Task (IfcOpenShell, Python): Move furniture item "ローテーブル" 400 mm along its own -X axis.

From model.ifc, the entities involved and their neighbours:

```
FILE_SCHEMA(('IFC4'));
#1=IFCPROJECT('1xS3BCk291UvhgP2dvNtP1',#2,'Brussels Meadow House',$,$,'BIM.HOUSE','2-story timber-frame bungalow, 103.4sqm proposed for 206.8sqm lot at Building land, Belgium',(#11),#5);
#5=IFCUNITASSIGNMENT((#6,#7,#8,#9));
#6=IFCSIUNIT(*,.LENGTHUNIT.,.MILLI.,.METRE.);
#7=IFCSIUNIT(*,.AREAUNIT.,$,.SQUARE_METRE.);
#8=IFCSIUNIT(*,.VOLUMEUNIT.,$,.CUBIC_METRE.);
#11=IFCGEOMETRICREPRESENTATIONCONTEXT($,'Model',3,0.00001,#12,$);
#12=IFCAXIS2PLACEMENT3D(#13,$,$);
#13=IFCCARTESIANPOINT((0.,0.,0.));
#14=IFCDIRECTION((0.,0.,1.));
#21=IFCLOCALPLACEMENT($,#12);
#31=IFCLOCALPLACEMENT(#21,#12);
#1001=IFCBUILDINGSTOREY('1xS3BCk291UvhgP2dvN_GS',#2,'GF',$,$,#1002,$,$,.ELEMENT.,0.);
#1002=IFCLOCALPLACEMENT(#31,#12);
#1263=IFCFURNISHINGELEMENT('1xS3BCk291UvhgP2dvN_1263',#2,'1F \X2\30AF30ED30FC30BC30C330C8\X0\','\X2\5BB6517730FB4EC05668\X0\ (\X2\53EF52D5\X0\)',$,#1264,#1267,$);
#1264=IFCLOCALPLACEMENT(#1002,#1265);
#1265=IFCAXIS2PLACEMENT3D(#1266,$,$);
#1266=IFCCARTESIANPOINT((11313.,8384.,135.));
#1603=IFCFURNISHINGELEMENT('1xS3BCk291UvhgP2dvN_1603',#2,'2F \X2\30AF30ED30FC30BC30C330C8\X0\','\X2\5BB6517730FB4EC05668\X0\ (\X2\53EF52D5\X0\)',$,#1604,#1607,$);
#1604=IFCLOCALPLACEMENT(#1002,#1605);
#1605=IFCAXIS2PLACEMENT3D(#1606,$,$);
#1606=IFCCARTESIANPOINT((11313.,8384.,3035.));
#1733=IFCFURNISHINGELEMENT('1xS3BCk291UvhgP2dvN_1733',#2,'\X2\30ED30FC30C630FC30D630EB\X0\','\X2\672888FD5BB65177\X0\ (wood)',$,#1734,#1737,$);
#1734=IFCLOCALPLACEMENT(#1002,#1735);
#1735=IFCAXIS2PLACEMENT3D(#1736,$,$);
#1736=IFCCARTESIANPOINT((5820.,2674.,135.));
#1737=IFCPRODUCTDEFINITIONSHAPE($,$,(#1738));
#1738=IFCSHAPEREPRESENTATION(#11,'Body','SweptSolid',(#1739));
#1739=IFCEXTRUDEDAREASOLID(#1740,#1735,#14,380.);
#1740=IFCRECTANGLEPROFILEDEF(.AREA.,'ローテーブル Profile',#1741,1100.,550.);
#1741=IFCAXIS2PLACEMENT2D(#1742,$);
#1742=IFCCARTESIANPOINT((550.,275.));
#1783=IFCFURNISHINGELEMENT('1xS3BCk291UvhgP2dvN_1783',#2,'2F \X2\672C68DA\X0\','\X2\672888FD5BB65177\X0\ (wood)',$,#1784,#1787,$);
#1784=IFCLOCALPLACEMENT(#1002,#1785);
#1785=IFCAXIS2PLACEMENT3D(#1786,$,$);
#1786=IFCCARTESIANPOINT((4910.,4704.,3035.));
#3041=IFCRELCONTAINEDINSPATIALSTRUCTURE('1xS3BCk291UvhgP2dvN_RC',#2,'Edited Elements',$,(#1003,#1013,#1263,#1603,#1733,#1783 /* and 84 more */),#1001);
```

```python
import ifcopenshell
import ifcopenshell.api.geometry
import ifcopenshell.util.placement

model = ifcopenshell.open("model.ifc")

item = model.by_guid("1xS3BCk291UvhgP2dvN_1733")
matrix = ifcopenshell.util.placement.get_local_placement(item.ObjectPlacement)
matrix[:3, 3] -= matrix[:3, 0] * 400.0
ifcopenshell.api.geometry.edit_object_placement(model, product=item, matrix=matrix, is_si=False)

print(ifcopenshell.util.placement.get_local_placement(item.ObjectPlacement).round(3) + 0.0)

model.write("model_v2.ifc")
```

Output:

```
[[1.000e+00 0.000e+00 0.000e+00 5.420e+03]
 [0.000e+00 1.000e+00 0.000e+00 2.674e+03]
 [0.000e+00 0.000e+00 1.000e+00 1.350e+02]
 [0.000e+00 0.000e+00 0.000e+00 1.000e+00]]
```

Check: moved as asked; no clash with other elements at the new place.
